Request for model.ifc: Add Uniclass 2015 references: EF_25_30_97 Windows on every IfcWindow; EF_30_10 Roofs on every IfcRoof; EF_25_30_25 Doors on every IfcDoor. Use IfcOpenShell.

First a look at what the model holds.

```python
import ifcopenshell

model = ifcopenshell.open("model.ifc")
print(model.schema)
print("classifications:", [c.Name for c in model.by_type("IfcClassification")])
for ifc_class in ("IfcDoor", "IfcRoof", "IfcStair", "IfcWall", "IfcWindow"):
    print(ifc_class, len(model.by_type(ifc_class)))
```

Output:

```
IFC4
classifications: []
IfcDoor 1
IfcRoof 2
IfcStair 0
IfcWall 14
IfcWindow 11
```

```python
import ifcopenshell
import ifcopenshell.api.classification

model = ifcopenshell.open("model.ifc")

system = ifcopenshell.api.classification.add_classification(model, classification="Uniclass 2015")

codes = {
    "IfcWindow": ("EF_25_30_97", "Windows"),
    "IfcRoof": ("EF_30_10", "Roofs"),
    "IfcDoor": ("EF_25_30_25", "Doors"),
}
for ifc_class, (code, name) in codes.items():
    products = model.by_type(ifc_class)
    ifcopenshell.api.classification.add_reference(
        model, products=products, classification=system, identification=code, name=name
    )
    print(code, len(products))

model.write("model-out.ifc")
```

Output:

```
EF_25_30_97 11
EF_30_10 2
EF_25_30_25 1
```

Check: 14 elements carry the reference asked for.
